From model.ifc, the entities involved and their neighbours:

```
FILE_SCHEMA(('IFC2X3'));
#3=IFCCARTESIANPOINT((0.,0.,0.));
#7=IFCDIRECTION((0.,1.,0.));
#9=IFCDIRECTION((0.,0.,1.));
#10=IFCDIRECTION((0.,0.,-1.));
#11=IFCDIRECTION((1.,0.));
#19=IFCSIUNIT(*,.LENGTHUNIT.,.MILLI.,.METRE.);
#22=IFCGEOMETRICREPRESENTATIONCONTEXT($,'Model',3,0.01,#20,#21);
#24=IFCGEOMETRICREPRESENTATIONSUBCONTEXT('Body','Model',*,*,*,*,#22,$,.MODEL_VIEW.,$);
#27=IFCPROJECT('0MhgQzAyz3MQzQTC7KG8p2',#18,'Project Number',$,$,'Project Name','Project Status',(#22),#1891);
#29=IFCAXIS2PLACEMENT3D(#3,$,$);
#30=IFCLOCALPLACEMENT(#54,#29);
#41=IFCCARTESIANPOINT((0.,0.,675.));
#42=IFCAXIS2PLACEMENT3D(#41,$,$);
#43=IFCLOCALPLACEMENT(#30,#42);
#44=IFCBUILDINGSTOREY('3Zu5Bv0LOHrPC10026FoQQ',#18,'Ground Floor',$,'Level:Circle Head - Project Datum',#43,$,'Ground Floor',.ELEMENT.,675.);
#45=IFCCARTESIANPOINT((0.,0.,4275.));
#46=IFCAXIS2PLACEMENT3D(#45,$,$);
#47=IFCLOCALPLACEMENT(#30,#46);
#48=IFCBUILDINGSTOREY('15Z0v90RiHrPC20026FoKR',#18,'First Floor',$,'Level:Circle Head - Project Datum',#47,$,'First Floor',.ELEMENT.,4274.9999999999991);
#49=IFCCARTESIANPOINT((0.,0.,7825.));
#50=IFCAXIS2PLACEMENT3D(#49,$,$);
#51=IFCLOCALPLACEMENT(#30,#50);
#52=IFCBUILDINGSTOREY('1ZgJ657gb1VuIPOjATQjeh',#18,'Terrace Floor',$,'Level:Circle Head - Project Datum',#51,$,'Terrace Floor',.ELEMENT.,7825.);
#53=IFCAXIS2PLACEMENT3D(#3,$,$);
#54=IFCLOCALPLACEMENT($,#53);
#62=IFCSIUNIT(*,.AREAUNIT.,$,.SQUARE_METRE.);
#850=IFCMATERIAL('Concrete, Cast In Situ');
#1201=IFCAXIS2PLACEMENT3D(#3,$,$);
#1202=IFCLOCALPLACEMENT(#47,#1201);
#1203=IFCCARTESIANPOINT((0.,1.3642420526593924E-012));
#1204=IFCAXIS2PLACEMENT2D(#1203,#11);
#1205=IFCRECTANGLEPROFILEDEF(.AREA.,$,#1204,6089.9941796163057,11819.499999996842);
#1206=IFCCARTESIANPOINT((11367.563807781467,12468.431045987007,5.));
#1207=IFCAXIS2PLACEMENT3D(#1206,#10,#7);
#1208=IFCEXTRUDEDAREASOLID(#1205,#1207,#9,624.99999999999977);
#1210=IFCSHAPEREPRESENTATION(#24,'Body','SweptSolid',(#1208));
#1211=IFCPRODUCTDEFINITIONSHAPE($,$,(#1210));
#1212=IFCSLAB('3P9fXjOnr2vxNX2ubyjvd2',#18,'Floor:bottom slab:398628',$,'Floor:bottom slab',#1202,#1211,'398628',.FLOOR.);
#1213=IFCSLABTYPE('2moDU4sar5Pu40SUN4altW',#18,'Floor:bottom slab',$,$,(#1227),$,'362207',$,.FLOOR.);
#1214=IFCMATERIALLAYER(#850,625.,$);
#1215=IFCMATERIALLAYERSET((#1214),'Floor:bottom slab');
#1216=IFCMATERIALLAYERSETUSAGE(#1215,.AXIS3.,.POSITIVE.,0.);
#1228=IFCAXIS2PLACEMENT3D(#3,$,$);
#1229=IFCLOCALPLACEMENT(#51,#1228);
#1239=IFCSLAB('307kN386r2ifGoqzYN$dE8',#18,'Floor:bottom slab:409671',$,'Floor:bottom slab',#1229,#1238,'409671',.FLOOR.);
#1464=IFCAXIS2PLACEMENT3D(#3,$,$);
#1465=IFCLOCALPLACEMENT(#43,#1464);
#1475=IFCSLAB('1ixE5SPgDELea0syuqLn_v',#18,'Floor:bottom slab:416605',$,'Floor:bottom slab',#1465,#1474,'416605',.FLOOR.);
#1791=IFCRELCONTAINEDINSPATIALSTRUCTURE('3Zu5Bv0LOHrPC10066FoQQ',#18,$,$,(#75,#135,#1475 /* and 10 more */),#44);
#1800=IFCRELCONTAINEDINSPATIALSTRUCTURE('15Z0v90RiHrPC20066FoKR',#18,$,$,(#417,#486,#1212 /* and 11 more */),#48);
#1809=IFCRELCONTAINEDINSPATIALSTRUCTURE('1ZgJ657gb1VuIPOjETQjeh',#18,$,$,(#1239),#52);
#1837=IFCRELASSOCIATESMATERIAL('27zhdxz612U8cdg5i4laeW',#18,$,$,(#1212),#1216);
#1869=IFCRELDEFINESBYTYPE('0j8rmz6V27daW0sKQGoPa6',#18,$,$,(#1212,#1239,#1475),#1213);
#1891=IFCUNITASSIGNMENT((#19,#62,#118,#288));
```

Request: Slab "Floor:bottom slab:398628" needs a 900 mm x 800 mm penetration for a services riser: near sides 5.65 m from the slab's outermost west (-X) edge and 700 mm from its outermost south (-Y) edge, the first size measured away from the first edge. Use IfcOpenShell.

```python
import numpy as np
import ifcopenshell
import ifcopenshell.api.feature
import ifcopenshell.api.geometry
import ifcopenshell.api.root
import ifcopenshell.geom
import ifcopenshell.util.placement
import ifcopenshell.util.representation
import ifcopenshell.util.shape
import ifcopenshell.util.unit

model = ifcopenshell.open("model.ifc")
unit_scale = ifcopenshell.util.unit.calculate_unit_scale(model)
settings = ifcopenshell.geom.settings()


def volume(element):
    """Net volume in cubic metres, openings subtracted."""
    shape = ifcopenshell.geom.create_shape(settings, element)
    return ifcopenshell.util.shape.get_volume(shape.geometry)


slab = model.by_id(1212)
before = volume(slab)

# Extent in the slab's own axes, in metres. The edges named are its -X and -Y sides.
slab_shape = ifcopenshell.geom.create_shape(settings, slab)
vertices = ifcopenshell.util.shape.get_vertices(slab_shape.geometry)
x_min, y_min, bottom = vertices.min(axis=0)
top = vertices[:, 2].max()

opening = ifcopenshell.api.root.create_entity(model, ifc_class="IfcOpeningElement", name="Services riser opening")
context = ifcopenshell.util.representation.get_context(model, "Model", "Body", "MODEL_VIEW")
width, depth = 0.9, 0.8
outline = [(0.0, 0.0), (width, 0.0), (width, depth), (0.0, depth), (0.0, 0.0)]
# Overshoot both faces by 50 mm so the cut is clean.
shape = ifcopenshell.api.geometry.add_slab_representation(
    model, context=context, depth=top - bottom + 0.1, polyline=outline
)
ifcopenshell.api.geometry.assign_representation(model, product=opening, representation=shape)

matrix = ifcopenshell.util.placement.get_local_placement(slab.ObjectPlacement)
matrix[:, 3] = matrix @ np.append(np.array([x_min + 5.65, y_min + 0.7, bottom - 0.05]) / unit_scale, 1.0)
ifcopenshell.api.geometry.edit_object_placement(model, product=opening, matrix=matrix, is_si=False)
ifcopenshell.api.feature.add_feature(model, feature=opening, element=slab)

after = volume(slab)

print(f"slab volume {before:.3f} -> {after:.3f} m3")

model.write("model_v2.ifc")
```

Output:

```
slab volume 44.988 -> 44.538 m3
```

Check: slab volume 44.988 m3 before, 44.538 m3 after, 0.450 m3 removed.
